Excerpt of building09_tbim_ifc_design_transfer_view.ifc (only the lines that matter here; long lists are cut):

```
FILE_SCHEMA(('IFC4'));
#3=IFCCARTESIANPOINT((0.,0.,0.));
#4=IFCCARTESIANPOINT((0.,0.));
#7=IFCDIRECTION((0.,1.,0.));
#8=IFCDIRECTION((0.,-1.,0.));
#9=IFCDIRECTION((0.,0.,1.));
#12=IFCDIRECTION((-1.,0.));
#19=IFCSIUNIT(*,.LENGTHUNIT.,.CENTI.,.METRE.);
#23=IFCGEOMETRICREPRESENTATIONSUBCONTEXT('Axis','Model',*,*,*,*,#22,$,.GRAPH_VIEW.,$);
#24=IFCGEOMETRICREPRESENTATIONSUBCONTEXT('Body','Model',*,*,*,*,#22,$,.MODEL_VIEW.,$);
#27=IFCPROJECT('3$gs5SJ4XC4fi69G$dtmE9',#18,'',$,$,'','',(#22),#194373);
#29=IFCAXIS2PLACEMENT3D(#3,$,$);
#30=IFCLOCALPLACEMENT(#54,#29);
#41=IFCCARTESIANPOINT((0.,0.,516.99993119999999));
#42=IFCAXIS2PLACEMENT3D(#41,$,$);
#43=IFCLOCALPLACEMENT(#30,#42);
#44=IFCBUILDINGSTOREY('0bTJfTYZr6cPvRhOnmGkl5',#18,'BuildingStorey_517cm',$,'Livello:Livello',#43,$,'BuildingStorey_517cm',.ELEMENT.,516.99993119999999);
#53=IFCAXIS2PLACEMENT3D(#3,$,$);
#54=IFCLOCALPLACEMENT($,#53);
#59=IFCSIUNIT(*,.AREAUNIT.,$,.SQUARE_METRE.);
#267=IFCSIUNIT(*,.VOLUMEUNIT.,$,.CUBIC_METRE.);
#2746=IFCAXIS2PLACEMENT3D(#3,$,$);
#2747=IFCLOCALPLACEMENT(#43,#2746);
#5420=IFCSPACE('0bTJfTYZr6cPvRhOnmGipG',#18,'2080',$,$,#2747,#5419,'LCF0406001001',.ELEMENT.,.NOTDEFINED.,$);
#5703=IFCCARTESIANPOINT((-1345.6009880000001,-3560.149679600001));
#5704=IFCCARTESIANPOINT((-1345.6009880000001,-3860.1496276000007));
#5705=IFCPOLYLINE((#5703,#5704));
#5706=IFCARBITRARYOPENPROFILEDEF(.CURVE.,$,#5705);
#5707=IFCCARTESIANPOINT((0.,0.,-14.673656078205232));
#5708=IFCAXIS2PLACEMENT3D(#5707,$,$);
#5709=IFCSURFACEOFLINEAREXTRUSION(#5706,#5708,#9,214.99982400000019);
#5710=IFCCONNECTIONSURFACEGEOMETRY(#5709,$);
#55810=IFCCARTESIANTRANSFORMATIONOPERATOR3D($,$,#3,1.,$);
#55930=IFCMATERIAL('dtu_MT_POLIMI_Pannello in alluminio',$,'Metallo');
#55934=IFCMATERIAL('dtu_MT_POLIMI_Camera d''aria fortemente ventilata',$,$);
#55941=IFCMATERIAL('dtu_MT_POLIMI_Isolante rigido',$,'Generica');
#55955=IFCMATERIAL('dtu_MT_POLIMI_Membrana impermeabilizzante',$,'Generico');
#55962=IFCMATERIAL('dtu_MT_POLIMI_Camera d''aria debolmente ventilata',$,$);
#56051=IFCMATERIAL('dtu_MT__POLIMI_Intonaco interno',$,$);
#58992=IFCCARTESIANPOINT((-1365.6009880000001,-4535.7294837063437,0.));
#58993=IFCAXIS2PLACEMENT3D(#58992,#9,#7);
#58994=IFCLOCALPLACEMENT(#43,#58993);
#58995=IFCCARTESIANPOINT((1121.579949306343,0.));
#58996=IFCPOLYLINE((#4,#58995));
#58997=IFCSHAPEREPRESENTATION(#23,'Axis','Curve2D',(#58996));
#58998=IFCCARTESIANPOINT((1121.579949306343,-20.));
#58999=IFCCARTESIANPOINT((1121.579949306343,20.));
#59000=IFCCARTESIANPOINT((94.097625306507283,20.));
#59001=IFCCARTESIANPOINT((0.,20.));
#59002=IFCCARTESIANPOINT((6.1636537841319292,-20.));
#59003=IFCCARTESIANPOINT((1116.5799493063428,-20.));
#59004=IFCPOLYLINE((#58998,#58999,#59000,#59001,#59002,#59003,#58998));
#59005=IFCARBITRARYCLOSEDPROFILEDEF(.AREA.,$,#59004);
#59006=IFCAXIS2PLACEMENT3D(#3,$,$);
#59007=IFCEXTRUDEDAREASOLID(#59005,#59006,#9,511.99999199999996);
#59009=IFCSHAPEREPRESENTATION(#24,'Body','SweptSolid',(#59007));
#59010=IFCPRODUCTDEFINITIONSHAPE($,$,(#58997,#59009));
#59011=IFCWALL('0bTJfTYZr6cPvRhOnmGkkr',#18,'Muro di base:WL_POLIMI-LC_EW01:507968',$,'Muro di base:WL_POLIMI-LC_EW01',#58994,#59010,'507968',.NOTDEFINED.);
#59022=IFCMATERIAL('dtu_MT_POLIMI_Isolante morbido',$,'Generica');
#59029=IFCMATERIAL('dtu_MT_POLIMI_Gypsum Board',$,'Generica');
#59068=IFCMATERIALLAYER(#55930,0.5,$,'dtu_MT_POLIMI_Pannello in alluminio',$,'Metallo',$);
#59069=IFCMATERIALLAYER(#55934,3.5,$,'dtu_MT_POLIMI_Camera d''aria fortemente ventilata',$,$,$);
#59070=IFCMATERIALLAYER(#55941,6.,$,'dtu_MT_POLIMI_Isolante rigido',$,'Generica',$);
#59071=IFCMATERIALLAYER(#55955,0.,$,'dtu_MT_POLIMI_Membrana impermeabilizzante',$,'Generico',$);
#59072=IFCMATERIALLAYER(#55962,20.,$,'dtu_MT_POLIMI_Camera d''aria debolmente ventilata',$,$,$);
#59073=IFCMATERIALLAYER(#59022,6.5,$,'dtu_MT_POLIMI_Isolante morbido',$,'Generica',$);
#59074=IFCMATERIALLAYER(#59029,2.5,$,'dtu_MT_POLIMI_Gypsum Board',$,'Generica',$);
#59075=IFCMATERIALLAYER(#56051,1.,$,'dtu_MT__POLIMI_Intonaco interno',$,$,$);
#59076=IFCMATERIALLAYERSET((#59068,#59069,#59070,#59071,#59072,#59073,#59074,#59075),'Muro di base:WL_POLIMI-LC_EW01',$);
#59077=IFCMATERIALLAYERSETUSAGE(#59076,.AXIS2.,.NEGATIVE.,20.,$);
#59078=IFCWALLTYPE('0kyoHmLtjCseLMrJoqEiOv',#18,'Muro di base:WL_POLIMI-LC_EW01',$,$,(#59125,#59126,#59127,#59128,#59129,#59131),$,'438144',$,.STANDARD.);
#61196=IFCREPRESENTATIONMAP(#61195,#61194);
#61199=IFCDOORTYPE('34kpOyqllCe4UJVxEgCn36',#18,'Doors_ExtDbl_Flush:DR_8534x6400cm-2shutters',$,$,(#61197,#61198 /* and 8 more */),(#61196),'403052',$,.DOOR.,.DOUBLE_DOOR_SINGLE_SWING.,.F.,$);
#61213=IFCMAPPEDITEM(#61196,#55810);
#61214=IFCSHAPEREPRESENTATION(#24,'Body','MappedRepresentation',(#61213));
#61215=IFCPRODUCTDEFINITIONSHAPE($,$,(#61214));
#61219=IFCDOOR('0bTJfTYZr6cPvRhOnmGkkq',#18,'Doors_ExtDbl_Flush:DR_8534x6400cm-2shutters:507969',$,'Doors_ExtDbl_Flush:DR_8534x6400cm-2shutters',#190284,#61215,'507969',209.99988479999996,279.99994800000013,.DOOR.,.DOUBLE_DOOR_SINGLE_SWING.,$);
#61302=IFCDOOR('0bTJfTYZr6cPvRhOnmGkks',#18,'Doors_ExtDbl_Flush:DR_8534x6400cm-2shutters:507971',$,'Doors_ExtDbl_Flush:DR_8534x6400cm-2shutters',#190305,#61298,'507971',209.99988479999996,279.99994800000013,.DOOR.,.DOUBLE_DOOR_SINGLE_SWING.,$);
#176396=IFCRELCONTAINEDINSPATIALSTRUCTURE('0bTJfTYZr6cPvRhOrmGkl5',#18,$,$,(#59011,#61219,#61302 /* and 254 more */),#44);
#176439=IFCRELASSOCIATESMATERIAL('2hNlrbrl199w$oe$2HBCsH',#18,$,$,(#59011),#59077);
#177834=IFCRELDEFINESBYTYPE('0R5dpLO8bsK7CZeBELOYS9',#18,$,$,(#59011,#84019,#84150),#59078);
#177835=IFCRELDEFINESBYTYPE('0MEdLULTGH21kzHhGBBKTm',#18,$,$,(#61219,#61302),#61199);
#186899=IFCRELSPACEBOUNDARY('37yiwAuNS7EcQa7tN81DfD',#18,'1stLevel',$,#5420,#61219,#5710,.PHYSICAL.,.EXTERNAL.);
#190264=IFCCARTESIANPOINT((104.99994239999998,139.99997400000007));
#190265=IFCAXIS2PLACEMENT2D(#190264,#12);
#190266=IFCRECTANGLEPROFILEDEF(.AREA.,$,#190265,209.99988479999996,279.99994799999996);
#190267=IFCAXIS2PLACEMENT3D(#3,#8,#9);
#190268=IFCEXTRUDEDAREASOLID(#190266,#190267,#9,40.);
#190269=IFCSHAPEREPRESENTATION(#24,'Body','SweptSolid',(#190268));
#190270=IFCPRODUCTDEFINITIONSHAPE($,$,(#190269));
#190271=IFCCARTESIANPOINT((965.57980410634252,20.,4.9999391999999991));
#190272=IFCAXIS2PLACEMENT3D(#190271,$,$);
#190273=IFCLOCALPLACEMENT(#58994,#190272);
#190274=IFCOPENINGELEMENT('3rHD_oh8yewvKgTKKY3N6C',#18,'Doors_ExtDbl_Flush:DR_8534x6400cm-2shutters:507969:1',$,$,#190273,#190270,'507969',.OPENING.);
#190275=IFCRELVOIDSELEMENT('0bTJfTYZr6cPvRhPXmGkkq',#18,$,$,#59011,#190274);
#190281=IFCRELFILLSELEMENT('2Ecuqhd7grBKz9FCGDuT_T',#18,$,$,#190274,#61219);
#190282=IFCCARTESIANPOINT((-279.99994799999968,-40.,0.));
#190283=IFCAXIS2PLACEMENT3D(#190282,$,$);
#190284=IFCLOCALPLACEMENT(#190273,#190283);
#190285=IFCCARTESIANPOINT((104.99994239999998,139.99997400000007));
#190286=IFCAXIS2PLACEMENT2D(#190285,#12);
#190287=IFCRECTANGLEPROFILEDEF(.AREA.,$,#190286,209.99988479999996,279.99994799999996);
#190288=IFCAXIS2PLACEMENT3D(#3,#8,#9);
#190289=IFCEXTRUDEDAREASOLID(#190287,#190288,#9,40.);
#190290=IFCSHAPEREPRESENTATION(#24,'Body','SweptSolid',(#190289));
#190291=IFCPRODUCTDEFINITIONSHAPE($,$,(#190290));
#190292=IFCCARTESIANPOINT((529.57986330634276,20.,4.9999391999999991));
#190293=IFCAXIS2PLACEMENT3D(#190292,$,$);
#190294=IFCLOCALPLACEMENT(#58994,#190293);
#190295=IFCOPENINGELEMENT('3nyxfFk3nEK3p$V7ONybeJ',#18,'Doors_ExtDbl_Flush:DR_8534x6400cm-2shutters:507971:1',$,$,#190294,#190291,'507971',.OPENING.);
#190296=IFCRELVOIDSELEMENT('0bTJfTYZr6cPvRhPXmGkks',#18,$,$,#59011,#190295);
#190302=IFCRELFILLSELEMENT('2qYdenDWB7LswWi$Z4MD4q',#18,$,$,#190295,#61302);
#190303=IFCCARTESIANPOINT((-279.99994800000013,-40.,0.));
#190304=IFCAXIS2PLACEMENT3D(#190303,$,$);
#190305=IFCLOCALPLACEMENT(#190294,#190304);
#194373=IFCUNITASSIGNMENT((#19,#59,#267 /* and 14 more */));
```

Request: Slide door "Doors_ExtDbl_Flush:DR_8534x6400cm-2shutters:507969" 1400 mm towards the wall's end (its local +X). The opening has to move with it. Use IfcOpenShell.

```python
import numpy as np
import ifcopenshell
import ifcopenshell.api.geometry
import ifcopenshell.util.placement
import ifcopenshell.util.unit

model = ifcopenshell.open("building09_tbim_ifc_design_transfer_view.ifc")
unit_scale = ifcopenshell.util.unit.calculate_unit_scale(model)

door = model.by_guid("0bTJfTYZr6cPvRhOnmGkkq")
opening = door.FillsVoids[0].RelatingOpeningElement
wall = opening.VoidsElements[0].RelatingBuildingElement

wall_matrix = ifcopenshell.util.placement.get_local_placement(wall.ObjectPlacement)
shift = wall_matrix[:3, 0] * 1.4 / unit_scale
before = ifcopenshell.util.placement.get_local_placement(door.ObjectPlacement)[:3, 3].copy()

# The door is placed relative to its opening, so it follows when the opening moves.
matrix = ifcopenshell.util.placement.get_local_placement(opening.ObjectPlacement)
matrix[:3, 3] += shift
ifcopenshell.api.geometry.edit_object_placement(
    model, product=opening, matrix=matrix, is_si=False, should_transform_children=True
)

# Space boundary surfaces are stored in each space's coordinates; move them too.
for rel in door.ProvidesBoundaries:
    if not rel.ConnectionGeometry:
        continue
    surface = rel.ConnectionGeometry.SurfaceOnRelatingElement
    space_matrix = ifcopenshell.util.placement.get_local_placement(rel.RelatingSpace.ObjectPlacement)
    point = np.array(surface.Position.Location.Coordinates) + space_matrix[:3, :3].T @ shift
    surface.Position = model.createIfcAxis2Placement3D(
        model.createIfcCartesianPoint(point.tolist()), surface.Position.Axis, surface.Position.RefDirection
    )

after = ifcopenshell.util.placement.get_local_placement(door.ObjectPlacement)[:3, 3]
print("door moved by", (after - before).round(3) + 0.0)

model.write("building09_tbim_ifc_design_transfer_view_v2.ifc")
```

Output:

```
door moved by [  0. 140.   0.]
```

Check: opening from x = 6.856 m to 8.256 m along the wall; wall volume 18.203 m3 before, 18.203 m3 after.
